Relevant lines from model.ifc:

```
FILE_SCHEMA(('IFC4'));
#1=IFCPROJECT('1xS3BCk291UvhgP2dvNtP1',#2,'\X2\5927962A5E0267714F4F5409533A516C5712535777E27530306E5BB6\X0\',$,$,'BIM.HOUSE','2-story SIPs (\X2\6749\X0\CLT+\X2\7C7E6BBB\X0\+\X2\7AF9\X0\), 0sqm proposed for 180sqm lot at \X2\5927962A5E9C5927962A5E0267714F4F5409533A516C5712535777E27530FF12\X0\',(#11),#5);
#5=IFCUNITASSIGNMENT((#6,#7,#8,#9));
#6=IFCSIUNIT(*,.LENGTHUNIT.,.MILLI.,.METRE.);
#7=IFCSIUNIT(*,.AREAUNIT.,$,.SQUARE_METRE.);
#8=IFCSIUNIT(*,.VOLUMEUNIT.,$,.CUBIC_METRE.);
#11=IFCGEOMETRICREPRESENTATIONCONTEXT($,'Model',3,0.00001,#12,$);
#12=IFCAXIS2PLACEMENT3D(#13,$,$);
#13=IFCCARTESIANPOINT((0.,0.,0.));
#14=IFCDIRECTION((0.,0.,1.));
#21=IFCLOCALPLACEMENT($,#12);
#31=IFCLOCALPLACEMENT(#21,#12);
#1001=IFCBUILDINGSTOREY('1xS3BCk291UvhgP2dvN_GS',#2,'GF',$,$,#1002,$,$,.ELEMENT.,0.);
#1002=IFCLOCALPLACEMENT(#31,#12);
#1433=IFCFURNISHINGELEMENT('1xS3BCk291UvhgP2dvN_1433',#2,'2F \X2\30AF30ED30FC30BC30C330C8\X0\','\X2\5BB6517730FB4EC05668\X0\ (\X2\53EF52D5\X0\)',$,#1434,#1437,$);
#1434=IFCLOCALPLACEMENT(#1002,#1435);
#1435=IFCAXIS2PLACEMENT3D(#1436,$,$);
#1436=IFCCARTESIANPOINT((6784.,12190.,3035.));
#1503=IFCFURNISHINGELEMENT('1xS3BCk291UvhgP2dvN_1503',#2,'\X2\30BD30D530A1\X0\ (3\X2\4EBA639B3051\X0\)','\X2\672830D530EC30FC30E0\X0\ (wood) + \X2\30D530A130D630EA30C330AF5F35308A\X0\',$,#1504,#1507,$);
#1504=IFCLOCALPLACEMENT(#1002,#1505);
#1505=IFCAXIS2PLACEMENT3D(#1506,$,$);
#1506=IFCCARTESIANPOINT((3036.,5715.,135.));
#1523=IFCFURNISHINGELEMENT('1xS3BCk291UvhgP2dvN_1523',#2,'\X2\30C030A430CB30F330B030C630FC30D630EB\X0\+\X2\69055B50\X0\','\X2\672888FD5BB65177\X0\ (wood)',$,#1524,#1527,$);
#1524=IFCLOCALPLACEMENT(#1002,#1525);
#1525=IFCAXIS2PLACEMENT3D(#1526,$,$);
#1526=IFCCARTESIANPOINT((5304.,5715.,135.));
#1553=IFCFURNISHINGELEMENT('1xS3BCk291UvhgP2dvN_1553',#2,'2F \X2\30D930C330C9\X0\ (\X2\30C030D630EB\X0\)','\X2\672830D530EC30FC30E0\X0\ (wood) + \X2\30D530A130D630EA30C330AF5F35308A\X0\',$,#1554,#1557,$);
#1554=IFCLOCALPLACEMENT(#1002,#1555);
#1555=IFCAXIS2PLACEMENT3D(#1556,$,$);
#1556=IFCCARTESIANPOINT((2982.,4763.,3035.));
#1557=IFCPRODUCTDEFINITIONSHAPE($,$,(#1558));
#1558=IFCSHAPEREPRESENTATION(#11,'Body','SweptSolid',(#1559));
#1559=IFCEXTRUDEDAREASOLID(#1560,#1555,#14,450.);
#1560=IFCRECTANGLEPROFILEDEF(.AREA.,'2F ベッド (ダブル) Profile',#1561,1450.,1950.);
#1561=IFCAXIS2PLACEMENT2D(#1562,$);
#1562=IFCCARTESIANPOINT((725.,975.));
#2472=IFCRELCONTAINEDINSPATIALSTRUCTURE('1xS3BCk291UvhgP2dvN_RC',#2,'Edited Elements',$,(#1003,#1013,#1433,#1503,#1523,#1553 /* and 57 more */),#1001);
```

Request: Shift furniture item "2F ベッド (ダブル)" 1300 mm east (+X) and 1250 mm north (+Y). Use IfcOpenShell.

```python
import ifcopenshell
import ifcopenshell.api.geometry
import ifcopenshell.util.placement

model = ifcopenshell.open("model.ifc")

item = model.by_guid("1xS3BCk291UvhgP2dvN_1553")
matrix = ifcopenshell.util.placement.get_local_placement(item.ObjectPlacement)
matrix[0, 3] += 1300.0
matrix[1, 3] += 1250.0
ifcopenshell.api.geometry.edit_object_placement(model, product=item, matrix=matrix, is_si=False)

print(ifcopenshell.util.placement.get_local_placement(item.ObjectPlacement).round(3) + 0.0)

model.write("model_v2.ifc")
```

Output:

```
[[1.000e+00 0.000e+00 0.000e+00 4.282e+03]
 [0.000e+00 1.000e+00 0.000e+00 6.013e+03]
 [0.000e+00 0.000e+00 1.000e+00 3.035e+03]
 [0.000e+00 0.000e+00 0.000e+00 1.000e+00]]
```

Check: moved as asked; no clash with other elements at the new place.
